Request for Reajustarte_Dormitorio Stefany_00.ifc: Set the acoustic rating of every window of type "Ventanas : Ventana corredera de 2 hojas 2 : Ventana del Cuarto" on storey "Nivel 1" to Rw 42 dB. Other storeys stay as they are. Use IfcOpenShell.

First a look at what the model holds.

```python
import ifcopenshell
import ifcopenshell.util.element

model = ifcopenshell.open("Reajustarte_Dormitorio Stefany_00.ifc")
print(model.schema)
storey = next(s for s in model.by_type("IfcBuildingStorey") if s.Name == "Nivel 1")
windows = [e for e in ifcopenshell.util.element.get_decomposition(storey) if e.is_a("IfcWindow")]
seen = {}
for e in windows:
    element_type = ifcopenshell.util.element.get_type(e)
    key = (element_type.Name if element_type != e and element_type else None, ifcopenshell.util.element.get_pset(e, "Pset_WindowCommon", "AcousticRating"))
    seen[key] = seen.get(key, 0) + 1
for (name, value), count in sorted(seen.items(), key=str):
    print(count, "x", name, "|", value)
```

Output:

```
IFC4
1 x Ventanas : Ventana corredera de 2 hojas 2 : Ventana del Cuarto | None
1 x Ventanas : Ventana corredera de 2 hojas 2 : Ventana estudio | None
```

```python
import ifcopenshell
import ifcopenshell.api.pset
import ifcopenshell.util.element

model = ifcopenshell.open("Reajustarte_Dormitorio Stefany_00.ifc")

storey = next(s for s in model.by_type("IfcBuildingStorey") if s.Name == "Nivel 1")
windows = [e for e in ifcopenshell.util.element.get_decomposition(storey) if e.is_a("IfcWindow")]

count = 0
for e in windows:
    element_type = ifcopenshell.util.element.get_type(e)
    if element_type in (None, e) or element_type.Name != "Ventanas : Ventana corredera de 2 hojas 2 : Ventana del Cuarto":
        continue
    # add_pset returns the element's existing set when there is one.
    pset = ifcopenshell.api.pset.add_pset(model, product=e, name="Pset_WindowCommon")
    ifcopenshell.api.pset.edit_pset(model, pset=pset, properties={"AcousticRating": "Rw 42 dB"})
    count += 1

print(count, "windows updated")

model.write("Reajustarte_Dormitorio Stefany_00_updated.ifc")
```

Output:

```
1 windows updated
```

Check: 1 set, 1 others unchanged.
